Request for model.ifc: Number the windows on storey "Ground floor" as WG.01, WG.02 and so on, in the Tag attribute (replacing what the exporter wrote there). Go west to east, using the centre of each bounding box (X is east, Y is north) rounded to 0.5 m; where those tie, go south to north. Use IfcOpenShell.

First a look at what the model holds.

```python
import ifcopenshell
import ifcopenshell.util.element
import ifcopenshell.util.placement

model = ifcopenshell.open("model.ifc")
print(model.schema)
storey = next(s for s in model.by_type("IfcBuildingStorey") if s.Name == "Ground floor")
windows = [e for e in ifcopenshell.util.element.get_decomposition(storey) if e.is_a("IfcWindow")]
for e in sorted(windows, key=lambda e: e.id()):
    origin = ifcopenshell.util.placement.get_local_placement(e.ObjectPlacement)[:3, 3]
    print(e.id(), e.Tag, e.Name, origin.round(2) + 0.0, sep=" | ")
```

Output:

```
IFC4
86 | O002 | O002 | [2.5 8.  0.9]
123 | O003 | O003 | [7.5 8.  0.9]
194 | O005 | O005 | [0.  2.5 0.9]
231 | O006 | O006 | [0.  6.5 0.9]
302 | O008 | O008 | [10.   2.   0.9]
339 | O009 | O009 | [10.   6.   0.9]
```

```python
import ifcopenshell
import ifcopenshell.geom
import ifcopenshell.util.element
import ifcopenshell.util.shape

model = ifcopenshell.open("model.ifc")
settings = ifcopenshell.geom.settings()
settings.set("use-world-coords", True)


def centre(element):
    shape = ifcopenshell.geom.create_shape(settings, element)
    return ifcopenshell.util.shape.get_bbox_centroid(shape.geometry)


storey = next(s for s in model.by_type("IfcBuildingStorey") if s.Name == "Ground floor")
windows = [e for e in ifcopenshell.util.element.get_decomposition(storey) if e.is_a("IfcWindow")]

# Insertion points can sit at a corner or the storey origin, so sort by the geometry (in metres).
centres = {e: centre(e) for e in windows}
windows.sort(key=lambda e: (round(centres[e][0] / 0.5), centres[e][1]))

for i, e in enumerate(windows, start=1):
    number = f"WG.{i:02d}"
    e.Tag = number
    print(e.id(), number)

model.write("model_rev.ifc")
```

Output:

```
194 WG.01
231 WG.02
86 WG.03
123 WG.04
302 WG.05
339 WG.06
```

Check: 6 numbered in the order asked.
